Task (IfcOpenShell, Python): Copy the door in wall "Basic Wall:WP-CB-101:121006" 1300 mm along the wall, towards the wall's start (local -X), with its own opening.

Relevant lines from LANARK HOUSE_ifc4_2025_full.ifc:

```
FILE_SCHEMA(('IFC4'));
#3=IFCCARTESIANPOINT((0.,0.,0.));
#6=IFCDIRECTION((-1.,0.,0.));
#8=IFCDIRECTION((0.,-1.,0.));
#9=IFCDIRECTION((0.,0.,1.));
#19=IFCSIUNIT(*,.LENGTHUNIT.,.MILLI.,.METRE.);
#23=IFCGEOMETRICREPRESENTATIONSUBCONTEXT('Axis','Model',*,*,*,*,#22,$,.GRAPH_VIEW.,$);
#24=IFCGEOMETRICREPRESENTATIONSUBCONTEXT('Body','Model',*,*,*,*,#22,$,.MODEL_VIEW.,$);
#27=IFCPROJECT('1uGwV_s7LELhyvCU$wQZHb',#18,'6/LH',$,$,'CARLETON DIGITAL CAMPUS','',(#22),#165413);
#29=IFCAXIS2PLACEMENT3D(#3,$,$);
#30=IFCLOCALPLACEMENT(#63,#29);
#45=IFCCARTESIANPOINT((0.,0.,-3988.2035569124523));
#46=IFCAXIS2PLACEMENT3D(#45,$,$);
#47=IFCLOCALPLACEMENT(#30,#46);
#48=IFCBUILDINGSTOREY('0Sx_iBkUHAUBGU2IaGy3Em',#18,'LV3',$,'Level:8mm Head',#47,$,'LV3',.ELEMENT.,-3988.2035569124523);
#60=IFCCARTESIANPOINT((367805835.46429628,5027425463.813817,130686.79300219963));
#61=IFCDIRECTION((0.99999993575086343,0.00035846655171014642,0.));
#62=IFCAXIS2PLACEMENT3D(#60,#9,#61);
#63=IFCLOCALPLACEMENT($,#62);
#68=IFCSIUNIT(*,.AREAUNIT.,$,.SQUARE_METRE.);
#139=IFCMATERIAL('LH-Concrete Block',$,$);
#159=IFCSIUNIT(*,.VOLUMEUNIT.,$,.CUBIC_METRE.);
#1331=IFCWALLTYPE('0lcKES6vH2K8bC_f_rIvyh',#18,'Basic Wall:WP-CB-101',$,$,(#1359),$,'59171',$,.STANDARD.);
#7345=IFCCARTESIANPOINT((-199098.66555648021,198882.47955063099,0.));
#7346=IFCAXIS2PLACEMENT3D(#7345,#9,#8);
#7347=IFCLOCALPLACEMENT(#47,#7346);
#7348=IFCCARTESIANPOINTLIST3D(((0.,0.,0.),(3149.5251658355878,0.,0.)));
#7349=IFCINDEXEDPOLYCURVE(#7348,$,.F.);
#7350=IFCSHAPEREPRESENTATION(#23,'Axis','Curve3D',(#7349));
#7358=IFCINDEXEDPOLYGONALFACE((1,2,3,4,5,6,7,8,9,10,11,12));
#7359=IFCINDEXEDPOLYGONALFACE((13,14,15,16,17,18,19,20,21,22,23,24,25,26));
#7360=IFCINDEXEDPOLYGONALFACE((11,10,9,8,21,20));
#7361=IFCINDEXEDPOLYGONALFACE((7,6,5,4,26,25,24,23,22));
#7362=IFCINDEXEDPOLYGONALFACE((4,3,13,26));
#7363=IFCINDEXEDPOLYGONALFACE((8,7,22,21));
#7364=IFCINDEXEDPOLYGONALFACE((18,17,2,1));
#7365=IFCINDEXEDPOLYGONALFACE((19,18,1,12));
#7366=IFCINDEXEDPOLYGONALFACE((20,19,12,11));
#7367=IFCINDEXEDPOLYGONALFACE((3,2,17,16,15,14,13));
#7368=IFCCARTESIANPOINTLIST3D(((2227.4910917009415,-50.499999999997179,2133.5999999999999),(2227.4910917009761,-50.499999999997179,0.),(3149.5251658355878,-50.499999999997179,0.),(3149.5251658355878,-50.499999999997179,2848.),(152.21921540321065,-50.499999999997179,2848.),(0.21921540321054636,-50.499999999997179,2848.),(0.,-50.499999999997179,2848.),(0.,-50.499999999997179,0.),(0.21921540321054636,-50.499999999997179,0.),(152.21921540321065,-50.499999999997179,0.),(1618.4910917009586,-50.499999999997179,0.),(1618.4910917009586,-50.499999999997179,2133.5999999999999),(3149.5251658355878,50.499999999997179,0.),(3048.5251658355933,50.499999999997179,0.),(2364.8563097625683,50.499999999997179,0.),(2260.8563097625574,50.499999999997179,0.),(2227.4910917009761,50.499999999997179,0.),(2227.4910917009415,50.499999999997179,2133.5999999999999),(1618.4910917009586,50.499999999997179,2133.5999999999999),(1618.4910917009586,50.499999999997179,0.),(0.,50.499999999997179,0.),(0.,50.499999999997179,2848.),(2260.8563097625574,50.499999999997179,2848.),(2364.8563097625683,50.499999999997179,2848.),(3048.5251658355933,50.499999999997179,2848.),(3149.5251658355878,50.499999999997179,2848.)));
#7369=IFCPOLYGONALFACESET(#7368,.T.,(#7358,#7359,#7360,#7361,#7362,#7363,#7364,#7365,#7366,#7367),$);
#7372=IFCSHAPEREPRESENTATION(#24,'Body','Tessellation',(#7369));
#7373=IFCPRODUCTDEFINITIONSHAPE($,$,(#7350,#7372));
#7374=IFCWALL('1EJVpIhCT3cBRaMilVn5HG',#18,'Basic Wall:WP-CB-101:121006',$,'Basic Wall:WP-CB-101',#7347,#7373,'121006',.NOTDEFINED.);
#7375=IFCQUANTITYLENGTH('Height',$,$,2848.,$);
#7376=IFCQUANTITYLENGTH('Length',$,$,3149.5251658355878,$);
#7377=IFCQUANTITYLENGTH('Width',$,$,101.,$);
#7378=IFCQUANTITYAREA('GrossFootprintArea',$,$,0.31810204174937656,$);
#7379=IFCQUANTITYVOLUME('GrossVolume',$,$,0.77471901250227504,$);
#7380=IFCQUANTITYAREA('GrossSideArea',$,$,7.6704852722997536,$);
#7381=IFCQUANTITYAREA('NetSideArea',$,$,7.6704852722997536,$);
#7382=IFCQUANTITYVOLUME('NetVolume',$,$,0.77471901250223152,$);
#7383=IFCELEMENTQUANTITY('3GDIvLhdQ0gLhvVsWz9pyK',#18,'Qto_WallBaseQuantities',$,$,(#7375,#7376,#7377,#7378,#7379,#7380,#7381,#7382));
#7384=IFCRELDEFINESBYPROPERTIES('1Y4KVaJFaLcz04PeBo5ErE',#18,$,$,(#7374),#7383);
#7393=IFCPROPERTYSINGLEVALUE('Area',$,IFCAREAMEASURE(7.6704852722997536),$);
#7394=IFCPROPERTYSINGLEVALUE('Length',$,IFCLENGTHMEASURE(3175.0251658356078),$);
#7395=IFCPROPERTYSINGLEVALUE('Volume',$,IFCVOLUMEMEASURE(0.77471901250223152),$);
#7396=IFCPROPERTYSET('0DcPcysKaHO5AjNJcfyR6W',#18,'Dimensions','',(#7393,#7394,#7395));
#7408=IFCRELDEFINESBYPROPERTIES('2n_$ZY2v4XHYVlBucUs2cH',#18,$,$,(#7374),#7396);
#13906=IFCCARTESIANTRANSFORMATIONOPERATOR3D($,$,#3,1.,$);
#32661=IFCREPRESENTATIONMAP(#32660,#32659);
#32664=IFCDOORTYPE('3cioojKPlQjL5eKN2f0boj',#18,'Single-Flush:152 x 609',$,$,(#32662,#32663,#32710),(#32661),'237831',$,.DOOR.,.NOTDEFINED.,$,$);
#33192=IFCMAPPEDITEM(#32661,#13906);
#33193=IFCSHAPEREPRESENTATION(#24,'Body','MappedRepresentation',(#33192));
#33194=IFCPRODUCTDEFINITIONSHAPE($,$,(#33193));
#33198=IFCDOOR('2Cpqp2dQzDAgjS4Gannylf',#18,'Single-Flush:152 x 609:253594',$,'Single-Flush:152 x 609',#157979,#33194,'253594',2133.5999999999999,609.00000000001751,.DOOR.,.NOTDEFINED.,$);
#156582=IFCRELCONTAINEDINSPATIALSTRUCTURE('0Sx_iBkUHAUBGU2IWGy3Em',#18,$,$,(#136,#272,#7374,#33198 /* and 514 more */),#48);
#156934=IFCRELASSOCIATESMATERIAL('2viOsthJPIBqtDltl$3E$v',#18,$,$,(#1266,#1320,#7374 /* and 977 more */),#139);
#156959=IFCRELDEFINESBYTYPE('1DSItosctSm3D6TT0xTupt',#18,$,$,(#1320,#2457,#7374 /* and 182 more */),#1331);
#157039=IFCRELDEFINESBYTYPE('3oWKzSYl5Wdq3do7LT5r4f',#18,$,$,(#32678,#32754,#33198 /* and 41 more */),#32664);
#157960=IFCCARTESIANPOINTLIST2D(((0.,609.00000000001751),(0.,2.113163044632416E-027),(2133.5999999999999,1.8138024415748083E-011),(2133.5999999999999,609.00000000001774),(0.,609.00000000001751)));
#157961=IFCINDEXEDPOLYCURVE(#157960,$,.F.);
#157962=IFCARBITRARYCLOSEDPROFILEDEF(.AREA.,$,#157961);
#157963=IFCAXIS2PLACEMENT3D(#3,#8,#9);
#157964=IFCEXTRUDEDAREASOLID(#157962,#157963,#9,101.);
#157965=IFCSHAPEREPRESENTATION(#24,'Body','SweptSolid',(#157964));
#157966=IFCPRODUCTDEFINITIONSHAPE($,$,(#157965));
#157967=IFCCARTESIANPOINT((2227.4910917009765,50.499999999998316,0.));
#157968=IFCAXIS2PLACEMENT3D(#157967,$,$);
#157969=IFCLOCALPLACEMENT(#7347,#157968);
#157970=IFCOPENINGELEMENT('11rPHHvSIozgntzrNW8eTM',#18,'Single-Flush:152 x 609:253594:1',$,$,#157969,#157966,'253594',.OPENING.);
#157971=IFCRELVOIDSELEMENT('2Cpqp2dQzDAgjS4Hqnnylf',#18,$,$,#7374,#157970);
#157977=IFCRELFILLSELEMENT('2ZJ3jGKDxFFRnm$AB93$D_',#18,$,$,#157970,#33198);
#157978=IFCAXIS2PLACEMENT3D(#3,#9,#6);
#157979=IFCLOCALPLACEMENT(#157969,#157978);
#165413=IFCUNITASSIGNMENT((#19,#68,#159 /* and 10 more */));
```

```python
import ifcopenshell
import ifcopenshell.api.feature
import ifcopenshell.api.geometry
import ifcopenshell.api.pset
import ifcopenshell.api.root
import ifcopenshell.geom
import ifcopenshell.util.element
import ifcopenshell.util.placement
import ifcopenshell.util.shape
import ifcopenshell.util.unit

model = ifcopenshell.open("LANARK HOUSE_ifc4_2025_full.ifc")
area_scale = ifcopenshell.util.unit.calculate_unit_scale(model, "AREAUNIT")
volume_scale = ifcopenshell.util.unit.calculate_unit_scale(model, "VOLUMEUNIT")
settings = ifcopenshell.geom.settings()


def volume(element):
    """Net volume in cubic metres, openings subtracted."""
    shape = ifcopenshell.geom.create_shape(settings, element)
    return ifcopenshell.util.shape.get_volume(shape.geometry)


def reuse_history(source, copy):
    """copy_class also copies each property set's owner history, people and application; keep the originals."""
    for rel in copy.IsDefinedBy:
        if rel.is_a("IfcRelDefinesByProperties") and (history := rel.RelatingPropertyDefinition.OwnerHistory):
            rel.RelatingPropertyDefinition.OwnerHistory = source.OwnerHistory
            ifcopenshell.util.element.remove_deep2(model, history)


door = model.by_guid("2Cpqp2dQzDAgjS4Gannylf")
opening = door.FillsVoids[0].RelatingOpeningElement
wall = opening.VoidsElements[0].RelatingBuildingElement
before = volume(wall)
shift = ifcopenshell.util.placement.get_local_placement(wall.ObjectPlacement)[:3, 0] * -1300.0

# copy_class copies the void relationship, type, container and properties, but no geometry.
new_opening = ifcopenshell.api.root.copy_class(model, product=opening)
new_opening.Representation = ifcopenshell.util.element.copy_deep(
    model, opening.Representation, exclude=["IfcGeometricRepresentationContext", "IfcRepresentationMap"]
)
new_opening.Name = "Single-Flush:152 x 609"
new_opening.Tag = None
reuse_history(opening, new_opening)
new_door = ifcopenshell.api.root.copy_class(model, product=door)
new_door.Representation = ifcopenshell.util.element.copy_deep(
    model, door.Representation, exclude=["IfcGeometricRepresentationContext", "IfcRepresentationMap"]
)
new_door.Name = "Single-Flush:152 x 609"
new_door.Tag = None
reuse_history(door, new_door)
ifcopenshell.api.feature.add_filling(model, opening=new_opening, element=new_door)

for old, new in ((opening, new_opening), (door, new_door)):
    matrix = ifcopenshell.util.placement.get_local_placement(old.ObjectPlacement)
    matrix[:3, 3] += shift
    ifcopenshell.api.geometry.edit_object_placement(model, product=new, matrix=matrix, is_si=False)

after = volume(wall)
thickness = 0.101  # wall thickness in metres

# Update the wall's stored quantities.
qto = model.by_id(ifcopenshell.util.element.get_pset(wall, "Qto_WallBaseQuantities", should_inherit=False)["id"])
ifcopenshell.api.pset.edit_qto(model, qto=qto, properties={
    "NetSideArea": after / thickness / area_scale,
    "NetVolume": after / volume_scale,
})
pset = model.by_id(ifcopenshell.util.element.get_pset(wall, "Dimensions", should_inherit=False)["id"])
ifcopenshell.api.pset.edit_pset(model, pset=pset, properties={
    "Area": model.create_entity("IfcAreaMeasure", after / thickness / area_scale),
    "Volume": model.create_entity("IfcVolumeMeasure", after / volume_scale),
})

print(f"wall volume {before:.3f} -> {after:.3f} m3")

model.write("LANARK HOUSE_ifc4_2025_full_edited.ifc")
```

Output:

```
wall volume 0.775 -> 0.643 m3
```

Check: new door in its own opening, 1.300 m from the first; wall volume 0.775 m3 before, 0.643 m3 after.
